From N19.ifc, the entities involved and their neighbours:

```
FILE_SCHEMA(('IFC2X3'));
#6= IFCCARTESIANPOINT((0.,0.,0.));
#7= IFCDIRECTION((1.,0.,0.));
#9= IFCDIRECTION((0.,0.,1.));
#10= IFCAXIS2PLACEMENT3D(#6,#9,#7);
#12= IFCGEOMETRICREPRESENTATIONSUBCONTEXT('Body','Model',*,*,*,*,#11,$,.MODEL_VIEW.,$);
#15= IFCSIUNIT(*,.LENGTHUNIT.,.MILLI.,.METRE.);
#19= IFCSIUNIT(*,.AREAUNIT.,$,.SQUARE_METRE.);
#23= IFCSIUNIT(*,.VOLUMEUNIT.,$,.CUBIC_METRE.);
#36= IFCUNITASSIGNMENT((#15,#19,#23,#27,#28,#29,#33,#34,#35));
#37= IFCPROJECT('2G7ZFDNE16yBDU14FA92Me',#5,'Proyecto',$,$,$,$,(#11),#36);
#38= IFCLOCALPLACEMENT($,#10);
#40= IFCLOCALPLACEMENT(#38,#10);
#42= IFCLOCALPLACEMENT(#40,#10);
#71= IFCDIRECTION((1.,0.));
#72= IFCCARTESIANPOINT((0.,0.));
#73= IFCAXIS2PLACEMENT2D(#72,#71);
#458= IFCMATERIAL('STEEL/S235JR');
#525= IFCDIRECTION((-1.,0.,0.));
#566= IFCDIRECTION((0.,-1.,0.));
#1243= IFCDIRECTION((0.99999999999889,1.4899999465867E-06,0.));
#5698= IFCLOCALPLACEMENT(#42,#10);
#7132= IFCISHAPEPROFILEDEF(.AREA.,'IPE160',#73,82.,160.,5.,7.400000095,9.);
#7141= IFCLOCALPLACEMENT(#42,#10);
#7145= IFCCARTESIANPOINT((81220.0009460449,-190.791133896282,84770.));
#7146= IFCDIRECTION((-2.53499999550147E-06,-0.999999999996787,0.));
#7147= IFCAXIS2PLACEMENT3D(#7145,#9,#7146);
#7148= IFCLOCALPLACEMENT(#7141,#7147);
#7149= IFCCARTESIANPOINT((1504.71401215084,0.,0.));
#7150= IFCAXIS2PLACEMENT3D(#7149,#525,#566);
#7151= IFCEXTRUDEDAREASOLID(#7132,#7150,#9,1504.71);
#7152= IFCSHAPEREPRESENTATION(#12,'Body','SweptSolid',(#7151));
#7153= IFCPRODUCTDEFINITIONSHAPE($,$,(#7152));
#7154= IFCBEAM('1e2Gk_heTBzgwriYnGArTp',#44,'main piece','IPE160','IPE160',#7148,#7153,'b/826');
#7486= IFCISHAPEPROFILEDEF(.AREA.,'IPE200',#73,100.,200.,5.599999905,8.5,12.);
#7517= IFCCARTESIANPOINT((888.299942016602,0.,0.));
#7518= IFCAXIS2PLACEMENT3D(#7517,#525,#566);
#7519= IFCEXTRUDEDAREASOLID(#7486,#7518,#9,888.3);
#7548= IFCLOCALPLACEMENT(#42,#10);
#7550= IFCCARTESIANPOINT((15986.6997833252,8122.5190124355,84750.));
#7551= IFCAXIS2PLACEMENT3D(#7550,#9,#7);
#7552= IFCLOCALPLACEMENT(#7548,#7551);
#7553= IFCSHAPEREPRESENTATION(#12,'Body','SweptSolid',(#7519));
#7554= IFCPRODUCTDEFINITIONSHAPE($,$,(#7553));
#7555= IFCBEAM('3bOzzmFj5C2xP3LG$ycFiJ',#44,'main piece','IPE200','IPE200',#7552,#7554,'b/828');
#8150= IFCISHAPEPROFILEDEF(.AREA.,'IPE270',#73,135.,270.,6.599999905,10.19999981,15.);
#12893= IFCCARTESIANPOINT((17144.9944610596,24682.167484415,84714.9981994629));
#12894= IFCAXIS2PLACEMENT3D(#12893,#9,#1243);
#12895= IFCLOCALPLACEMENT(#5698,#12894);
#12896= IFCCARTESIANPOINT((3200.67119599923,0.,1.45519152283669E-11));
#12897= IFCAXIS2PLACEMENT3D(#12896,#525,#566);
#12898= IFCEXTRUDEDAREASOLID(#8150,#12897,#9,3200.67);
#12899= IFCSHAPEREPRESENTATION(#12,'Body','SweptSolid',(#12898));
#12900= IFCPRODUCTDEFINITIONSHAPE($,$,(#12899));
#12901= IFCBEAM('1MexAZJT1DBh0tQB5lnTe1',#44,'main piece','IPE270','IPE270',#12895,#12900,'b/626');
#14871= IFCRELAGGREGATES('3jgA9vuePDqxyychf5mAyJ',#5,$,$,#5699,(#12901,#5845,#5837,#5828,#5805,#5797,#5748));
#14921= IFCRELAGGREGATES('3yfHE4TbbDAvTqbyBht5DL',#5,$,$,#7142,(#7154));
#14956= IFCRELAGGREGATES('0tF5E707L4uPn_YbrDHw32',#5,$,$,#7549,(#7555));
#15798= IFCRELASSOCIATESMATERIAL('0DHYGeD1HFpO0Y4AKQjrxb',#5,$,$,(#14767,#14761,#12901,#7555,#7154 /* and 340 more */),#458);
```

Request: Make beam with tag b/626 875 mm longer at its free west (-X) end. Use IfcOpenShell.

```python
import ifcopenshell
import ifcopenshell.util.representation

model = ifcopenshell.open("N19.ifc")

member = model.by_guid("1MexAZJT1DBh0tQB5lnTe1")
change = 875.0

# The extrusion runs towards the end named, so only its depth changes.
body = ifcopenshell.util.representation.get_representation(member, "Model", "Body")
solid = body.Items[0]
old_length = solid.Depth
solid.Depth += change

print(f"length {old_length:g} -> {solid.Depth:g}")

model.write("N19_updated.ifc")
```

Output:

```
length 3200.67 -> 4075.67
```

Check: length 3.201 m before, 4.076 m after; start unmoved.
